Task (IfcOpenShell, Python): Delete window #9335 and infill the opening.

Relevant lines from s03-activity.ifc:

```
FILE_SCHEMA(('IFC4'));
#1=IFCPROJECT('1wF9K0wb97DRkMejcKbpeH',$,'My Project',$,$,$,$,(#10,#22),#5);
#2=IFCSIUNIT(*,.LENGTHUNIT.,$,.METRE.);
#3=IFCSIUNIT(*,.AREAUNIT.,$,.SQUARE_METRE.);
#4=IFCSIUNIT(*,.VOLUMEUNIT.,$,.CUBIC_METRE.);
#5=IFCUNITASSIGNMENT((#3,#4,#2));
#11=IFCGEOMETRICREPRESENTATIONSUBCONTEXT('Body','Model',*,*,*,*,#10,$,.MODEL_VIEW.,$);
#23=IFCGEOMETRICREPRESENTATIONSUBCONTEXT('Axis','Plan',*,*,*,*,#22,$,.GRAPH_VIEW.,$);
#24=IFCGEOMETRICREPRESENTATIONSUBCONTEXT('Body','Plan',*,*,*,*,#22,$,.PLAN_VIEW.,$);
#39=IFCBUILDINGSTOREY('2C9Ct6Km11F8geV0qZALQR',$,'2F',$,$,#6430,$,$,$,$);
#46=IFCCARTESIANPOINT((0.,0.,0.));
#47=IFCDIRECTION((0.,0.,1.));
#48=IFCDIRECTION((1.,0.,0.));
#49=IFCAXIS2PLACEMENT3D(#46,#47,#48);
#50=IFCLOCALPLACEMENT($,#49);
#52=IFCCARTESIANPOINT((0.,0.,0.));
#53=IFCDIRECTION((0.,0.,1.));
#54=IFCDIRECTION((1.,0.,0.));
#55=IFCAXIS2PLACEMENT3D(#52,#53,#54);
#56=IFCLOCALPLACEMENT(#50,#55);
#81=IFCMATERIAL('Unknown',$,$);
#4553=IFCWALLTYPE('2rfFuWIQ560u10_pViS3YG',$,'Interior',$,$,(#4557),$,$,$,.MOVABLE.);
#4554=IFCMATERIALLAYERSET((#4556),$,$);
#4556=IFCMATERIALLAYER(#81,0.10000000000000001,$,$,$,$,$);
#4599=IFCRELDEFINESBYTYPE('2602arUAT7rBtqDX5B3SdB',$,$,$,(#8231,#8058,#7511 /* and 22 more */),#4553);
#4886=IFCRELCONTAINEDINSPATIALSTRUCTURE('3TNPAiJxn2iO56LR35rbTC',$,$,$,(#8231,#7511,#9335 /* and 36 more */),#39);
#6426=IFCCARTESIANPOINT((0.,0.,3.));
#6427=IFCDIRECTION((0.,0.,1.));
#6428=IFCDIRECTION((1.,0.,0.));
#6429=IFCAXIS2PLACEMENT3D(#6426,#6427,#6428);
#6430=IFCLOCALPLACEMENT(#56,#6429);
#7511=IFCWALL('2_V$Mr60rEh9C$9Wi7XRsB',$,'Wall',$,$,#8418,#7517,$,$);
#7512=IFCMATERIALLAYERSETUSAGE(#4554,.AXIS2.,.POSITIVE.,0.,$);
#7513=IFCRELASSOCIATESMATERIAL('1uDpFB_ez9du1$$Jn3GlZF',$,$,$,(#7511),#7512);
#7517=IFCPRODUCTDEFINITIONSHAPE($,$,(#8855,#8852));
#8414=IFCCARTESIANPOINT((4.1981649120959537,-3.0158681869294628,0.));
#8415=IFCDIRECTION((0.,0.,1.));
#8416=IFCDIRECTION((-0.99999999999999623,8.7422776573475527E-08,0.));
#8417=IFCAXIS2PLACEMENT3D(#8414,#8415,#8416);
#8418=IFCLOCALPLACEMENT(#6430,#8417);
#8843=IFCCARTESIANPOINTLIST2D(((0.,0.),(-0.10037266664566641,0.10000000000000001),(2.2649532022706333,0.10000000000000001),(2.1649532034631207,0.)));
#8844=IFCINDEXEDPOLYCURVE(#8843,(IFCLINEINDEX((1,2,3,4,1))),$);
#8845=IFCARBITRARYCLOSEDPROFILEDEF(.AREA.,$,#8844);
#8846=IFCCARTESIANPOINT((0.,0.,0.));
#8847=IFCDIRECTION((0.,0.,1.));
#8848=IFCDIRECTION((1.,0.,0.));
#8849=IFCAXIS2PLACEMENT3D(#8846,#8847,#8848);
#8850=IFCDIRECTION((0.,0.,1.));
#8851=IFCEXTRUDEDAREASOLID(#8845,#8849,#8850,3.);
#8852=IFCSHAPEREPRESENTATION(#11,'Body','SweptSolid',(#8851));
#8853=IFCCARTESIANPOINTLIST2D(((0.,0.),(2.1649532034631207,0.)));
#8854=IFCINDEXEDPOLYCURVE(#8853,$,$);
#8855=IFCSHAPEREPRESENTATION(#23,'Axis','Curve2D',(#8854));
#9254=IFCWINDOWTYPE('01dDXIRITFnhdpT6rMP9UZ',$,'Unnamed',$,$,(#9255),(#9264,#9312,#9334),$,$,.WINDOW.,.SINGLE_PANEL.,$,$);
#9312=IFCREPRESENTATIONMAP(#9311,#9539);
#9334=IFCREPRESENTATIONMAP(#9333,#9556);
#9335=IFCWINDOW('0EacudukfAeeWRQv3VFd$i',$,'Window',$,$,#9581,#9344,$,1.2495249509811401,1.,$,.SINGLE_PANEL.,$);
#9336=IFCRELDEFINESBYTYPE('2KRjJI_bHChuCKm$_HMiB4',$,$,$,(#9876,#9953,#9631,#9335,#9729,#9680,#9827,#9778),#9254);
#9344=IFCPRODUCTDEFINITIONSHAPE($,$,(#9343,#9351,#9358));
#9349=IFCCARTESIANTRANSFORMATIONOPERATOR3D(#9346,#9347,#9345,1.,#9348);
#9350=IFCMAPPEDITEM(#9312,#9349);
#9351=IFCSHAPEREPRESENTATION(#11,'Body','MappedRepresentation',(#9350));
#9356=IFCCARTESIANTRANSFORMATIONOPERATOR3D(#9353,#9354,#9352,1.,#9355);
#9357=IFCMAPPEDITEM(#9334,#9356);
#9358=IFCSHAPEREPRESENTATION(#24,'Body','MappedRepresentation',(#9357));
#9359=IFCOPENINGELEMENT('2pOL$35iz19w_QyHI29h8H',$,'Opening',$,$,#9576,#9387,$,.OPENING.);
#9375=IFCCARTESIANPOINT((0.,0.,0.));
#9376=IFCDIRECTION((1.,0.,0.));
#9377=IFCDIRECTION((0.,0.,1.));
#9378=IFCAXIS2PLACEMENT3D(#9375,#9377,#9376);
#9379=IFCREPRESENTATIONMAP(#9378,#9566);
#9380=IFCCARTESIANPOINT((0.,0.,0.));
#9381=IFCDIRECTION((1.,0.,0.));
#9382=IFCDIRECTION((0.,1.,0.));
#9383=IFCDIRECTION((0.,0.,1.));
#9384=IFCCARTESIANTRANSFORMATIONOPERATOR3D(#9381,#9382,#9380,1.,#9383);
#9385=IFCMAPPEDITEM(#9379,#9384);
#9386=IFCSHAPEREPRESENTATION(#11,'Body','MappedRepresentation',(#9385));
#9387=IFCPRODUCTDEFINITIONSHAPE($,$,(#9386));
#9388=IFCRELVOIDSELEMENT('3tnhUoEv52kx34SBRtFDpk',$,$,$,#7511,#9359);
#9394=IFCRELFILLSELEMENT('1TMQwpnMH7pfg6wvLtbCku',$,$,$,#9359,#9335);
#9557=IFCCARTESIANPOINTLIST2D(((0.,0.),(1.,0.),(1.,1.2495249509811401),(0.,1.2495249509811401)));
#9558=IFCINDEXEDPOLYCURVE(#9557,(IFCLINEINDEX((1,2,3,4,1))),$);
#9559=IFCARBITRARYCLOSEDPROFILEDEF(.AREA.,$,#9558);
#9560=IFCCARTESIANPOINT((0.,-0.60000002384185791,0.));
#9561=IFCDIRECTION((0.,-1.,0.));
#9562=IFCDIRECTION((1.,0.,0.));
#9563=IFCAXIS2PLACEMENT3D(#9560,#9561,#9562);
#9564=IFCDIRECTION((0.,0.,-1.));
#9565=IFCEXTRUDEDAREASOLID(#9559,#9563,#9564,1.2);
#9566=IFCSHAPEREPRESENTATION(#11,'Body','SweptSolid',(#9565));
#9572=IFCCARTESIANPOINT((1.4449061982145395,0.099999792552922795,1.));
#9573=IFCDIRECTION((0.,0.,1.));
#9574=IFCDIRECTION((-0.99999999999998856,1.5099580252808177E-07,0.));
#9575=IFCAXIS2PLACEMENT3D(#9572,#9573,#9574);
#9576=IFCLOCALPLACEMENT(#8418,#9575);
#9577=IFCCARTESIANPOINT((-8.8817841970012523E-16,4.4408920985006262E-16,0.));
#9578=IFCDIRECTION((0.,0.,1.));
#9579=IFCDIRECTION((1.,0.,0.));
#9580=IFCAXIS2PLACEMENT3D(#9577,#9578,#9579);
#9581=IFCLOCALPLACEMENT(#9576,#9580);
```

```python
import ifcopenshell
import ifcopenshell.api.feature
import ifcopenshell.api.root
import ifcopenshell.geom
import ifcopenshell.util.shape

model = ifcopenshell.open("s03-activity.ifc")
settings = ifcopenshell.geom.settings()


def volume(element):
    """Net volume in cubic metres, openings subtracted."""
    shape = ifcopenshell.geom.create_shape(settings, element)
    return ifcopenshell.util.shape.get_volume(shape.geometry)


window = model.by_guid("0EacudukfAeeWRQv3VFd$i")
opening = window.FillsVoids[0].RelatingOpeningElement
wall = opening.VoidsElements[0].RelatingBuildingElement
before = volume(wall)

ifcopenshell.api.root.remove_product(model, product=window)
ifcopenshell.api.feature.remove_feature(model, feature=opening)

after = volume(wall)

print(f"wall volume {before:.3f} -> {after:.3f} m3")

model.write("s03-activity_v2.ifc")
```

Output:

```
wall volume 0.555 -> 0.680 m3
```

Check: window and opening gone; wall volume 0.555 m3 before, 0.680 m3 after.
